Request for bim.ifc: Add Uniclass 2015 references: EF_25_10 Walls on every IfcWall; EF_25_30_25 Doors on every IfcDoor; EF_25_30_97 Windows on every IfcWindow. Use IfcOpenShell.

First a look at what the model holds.

```python
import ifcopenshell

model = ifcopenshell.open("bim.ifc")
print(model.schema)
print("classifications:", [c.Name for c in model.by_type("IfcClassification")])
for ifc_class in ("IfcDoor", "IfcRoof", "IfcStair", "IfcWall", "IfcWindow"):
    print(ifc_class, len(model.by_type(ifc_class)))
```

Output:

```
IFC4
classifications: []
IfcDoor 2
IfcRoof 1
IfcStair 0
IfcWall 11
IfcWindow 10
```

```python
import ifcopenshell
import ifcopenshell.api.classification

model = ifcopenshell.open("bim.ifc")

system = ifcopenshell.api.classification.add_classification(model, classification="Uniclass 2015")

codes = {
    "IfcWall": ("EF_25_10", "Walls"),
    "IfcDoor": ("EF_25_30_25", "Doors"),
    "IfcWindow": ("EF_25_30_97", "Windows"),
}
for ifc_class, (code, name) in codes.items():
    products = model.by_type(ifc_class)
    ifcopenshell.api.classification.add_reference(
        model, products=products, classification=system, identification=code, name=name
    )
    print(code, len(products))

model.write("bim_v2.ifc")
```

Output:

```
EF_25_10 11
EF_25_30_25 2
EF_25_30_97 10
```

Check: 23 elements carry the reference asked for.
